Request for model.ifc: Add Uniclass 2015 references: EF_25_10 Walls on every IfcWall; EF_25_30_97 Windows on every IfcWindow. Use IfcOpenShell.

First a look at what the model holds.

```python
import ifcopenshell

model = ifcopenshell.open("model.ifc")
print(model.schema)
print("classifications:", [c.Name for c in model.by_type("IfcClassification")])
for ifc_class in ("IfcDoor", "IfcRoof", "IfcStair", "IfcWall", "IfcWindow"):
    print(ifc_class, len(model.by_type(ifc_class)))
```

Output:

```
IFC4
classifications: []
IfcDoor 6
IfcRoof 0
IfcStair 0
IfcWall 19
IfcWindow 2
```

```python
import ifcopenshell
import ifcopenshell.api.classification

model = ifcopenshell.open("model.ifc")

system = ifcopenshell.api.classification.add_classification(model, classification="Uniclass 2015")

codes = {
    "IfcWall": ("EF_25_10", "Walls"),
    "IfcWindow": ("EF_25_30_97", "Windows"),
}
for ifc_class, (code, name) in codes.items():
    products = model.by_type(ifc_class)
    ifcopenshell.api.classification.add_reference(
        model, products=products, classification=system, identification=code, name=name
    )
    print(code, len(products))

model.write("model_v2.ifc")
```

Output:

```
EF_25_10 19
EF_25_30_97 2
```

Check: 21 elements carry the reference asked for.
